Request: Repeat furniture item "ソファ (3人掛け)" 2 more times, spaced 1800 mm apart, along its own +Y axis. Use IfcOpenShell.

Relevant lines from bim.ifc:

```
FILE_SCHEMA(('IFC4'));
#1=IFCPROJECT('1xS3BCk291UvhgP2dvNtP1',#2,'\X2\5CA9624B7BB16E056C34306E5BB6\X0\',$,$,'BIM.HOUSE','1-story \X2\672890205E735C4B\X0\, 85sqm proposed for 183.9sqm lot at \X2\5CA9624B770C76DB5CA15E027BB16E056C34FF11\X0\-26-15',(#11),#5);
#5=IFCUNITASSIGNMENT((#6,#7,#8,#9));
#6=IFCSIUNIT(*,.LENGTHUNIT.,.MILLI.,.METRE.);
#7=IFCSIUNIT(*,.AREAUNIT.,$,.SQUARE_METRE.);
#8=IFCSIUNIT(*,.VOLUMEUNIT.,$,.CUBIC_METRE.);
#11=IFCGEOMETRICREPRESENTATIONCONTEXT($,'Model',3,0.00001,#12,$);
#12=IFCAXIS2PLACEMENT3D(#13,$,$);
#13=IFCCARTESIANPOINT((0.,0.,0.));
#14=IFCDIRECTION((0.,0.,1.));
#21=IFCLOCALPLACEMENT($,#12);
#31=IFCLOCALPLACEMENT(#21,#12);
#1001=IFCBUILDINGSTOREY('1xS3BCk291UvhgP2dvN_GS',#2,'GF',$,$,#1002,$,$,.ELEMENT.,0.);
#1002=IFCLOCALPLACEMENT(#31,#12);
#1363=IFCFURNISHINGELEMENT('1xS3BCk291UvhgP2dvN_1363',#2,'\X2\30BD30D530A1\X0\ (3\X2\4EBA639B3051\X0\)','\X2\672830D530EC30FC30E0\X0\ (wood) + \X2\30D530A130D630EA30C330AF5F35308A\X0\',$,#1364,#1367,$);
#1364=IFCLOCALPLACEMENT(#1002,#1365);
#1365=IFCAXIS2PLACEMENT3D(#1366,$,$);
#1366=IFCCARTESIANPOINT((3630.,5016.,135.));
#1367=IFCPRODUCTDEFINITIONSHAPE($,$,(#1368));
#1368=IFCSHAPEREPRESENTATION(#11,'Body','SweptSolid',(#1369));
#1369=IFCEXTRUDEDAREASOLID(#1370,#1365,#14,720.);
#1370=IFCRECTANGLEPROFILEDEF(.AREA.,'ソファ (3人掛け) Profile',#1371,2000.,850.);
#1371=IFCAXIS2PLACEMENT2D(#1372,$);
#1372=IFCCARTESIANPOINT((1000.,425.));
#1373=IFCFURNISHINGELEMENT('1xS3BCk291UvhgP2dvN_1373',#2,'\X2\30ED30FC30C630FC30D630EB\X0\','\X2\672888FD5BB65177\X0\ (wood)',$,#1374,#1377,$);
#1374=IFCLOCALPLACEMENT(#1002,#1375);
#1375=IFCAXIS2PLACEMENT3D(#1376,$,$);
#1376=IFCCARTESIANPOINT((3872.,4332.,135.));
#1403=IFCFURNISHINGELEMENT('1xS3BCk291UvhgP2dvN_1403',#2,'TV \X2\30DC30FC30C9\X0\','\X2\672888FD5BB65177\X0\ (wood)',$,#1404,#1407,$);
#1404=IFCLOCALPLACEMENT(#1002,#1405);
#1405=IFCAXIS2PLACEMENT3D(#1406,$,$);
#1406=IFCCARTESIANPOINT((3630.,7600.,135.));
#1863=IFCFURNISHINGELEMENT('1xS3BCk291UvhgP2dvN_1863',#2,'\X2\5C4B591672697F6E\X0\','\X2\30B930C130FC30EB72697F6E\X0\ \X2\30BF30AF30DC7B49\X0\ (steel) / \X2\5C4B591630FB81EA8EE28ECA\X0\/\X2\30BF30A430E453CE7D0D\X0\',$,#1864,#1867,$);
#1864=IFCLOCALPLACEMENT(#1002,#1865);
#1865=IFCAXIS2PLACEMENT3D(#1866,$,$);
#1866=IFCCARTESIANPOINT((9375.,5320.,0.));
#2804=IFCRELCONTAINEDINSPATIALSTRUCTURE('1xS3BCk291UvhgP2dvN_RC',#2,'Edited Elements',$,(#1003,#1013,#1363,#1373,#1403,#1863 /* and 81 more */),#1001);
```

```python
import ifcopenshell
import ifcopenshell.api.geometry
import ifcopenshell.api.root
import ifcopenshell.util.element
import ifcopenshell.util.placement
import ifcopenshell.util.unit

model = ifcopenshell.open("bim.ifc")
unit_scale = ifcopenshell.util.unit.calculate_unit_scale(model)


def reuse_history(source, copy):
    """copy_class also copies each property set's owner history, people and application; keep the originals."""
    for rel in copy.IsDefinedBy:
        if rel.is_a("IfcRelDefinesByProperties") and (history := rel.RelatingPropertyDefinition.OwnerHistory):
            rel.RelatingPropertyDefinition.OwnerHistory = source.OwnerHistory
            ifcopenshell.util.element.remove_deep2(model, history)


source = model.by_id(1363)
base = ifcopenshell.util.placement.get_local_placement(source.ObjectPlacement)
step = base[:3, 1] * 1.8 / unit_scale

for i in range(1, 3):
    copy = ifcopenshell.api.root.copy_class(model, product=source)
    copy.Representation = ifcopenshell.util.element.copy_deep(
        model, source.Representation, exclude=["IfcGeometricRepresentationContext", "IfcRepresentationMap"]
    )
    reuse_history(source, copy)
    matrix = base.copy()
    matrix[:3, 3] += i * step
    print("added at", matrix[:3, 3].round(3) + 0.0)
    ifcopenshell.api.geometry.edit_object_placement(model, product=copy, matrix=matrix, is_si=False)

model.write("bim-out.ifc")
```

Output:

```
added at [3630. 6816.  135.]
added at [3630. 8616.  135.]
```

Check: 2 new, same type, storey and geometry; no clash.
